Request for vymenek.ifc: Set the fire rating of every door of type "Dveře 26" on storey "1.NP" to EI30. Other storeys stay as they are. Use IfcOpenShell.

First a look at what the model holds.

```python
import ifcopenshell
import ifcopenshell.util.element

model = ifcopenshell.open("vymenek.ifc")
print(model.schema)
storey = next(s for s in model.by_type("IfcBuildingStorey") if s.Name == "1.NP")
doors = [e for e in ifcopenshell.util.element.get_decomposition(storey) if e.is_a("IfcDoor")]
seen = {}
for e in doors:
    element_type = ifcopenshell.util.element.get_type(e)
    key = (element_type.Name if element_type != e and element_type else None, ifcopenshell.util.element.get_pset(e, "Pset_DoorCommon", "FireRating"))
    seen[key] = seen.get(key, 0) + 1
for (name, value), count in sorted(seen.items(), key=str):
    print(count, "x", name, "|", value)
```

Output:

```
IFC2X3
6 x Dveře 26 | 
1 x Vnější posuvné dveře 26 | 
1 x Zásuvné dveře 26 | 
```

```python
import ifcopenshell
import ifcopenshell.api.pset
import ifcopenshell.util.element

model = ifcopenshell.open("vymenek.ifc")

storey = next(s for s in model.by_type("IfcBuildingStorey") if s.Name == "1.NP")
doors = [e for e in ifcopenshell.util.element.get_decomposition(storey) if e.is_a("IfcDoor")]

count = 0
for e in doors:
    element_type = ifcopenshell.util.element.get_type(e)
    if element_type in (None, e) or element_type.Name != "Dveře 26":
        continue
    # add_pset returns the element's existing set when there is one.
    pset = ifcopenshell.api.pset.add_pset(model, product=e, name="Pset_DoorCommon")
    ifcopenshell.api.pset.edit_pset(model, pset=pset, properties={"FireRating": "EI30"})
    count += 1

print(count, "doors updated")

model.write("vymenek-out.ifc")
```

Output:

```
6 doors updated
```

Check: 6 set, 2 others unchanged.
